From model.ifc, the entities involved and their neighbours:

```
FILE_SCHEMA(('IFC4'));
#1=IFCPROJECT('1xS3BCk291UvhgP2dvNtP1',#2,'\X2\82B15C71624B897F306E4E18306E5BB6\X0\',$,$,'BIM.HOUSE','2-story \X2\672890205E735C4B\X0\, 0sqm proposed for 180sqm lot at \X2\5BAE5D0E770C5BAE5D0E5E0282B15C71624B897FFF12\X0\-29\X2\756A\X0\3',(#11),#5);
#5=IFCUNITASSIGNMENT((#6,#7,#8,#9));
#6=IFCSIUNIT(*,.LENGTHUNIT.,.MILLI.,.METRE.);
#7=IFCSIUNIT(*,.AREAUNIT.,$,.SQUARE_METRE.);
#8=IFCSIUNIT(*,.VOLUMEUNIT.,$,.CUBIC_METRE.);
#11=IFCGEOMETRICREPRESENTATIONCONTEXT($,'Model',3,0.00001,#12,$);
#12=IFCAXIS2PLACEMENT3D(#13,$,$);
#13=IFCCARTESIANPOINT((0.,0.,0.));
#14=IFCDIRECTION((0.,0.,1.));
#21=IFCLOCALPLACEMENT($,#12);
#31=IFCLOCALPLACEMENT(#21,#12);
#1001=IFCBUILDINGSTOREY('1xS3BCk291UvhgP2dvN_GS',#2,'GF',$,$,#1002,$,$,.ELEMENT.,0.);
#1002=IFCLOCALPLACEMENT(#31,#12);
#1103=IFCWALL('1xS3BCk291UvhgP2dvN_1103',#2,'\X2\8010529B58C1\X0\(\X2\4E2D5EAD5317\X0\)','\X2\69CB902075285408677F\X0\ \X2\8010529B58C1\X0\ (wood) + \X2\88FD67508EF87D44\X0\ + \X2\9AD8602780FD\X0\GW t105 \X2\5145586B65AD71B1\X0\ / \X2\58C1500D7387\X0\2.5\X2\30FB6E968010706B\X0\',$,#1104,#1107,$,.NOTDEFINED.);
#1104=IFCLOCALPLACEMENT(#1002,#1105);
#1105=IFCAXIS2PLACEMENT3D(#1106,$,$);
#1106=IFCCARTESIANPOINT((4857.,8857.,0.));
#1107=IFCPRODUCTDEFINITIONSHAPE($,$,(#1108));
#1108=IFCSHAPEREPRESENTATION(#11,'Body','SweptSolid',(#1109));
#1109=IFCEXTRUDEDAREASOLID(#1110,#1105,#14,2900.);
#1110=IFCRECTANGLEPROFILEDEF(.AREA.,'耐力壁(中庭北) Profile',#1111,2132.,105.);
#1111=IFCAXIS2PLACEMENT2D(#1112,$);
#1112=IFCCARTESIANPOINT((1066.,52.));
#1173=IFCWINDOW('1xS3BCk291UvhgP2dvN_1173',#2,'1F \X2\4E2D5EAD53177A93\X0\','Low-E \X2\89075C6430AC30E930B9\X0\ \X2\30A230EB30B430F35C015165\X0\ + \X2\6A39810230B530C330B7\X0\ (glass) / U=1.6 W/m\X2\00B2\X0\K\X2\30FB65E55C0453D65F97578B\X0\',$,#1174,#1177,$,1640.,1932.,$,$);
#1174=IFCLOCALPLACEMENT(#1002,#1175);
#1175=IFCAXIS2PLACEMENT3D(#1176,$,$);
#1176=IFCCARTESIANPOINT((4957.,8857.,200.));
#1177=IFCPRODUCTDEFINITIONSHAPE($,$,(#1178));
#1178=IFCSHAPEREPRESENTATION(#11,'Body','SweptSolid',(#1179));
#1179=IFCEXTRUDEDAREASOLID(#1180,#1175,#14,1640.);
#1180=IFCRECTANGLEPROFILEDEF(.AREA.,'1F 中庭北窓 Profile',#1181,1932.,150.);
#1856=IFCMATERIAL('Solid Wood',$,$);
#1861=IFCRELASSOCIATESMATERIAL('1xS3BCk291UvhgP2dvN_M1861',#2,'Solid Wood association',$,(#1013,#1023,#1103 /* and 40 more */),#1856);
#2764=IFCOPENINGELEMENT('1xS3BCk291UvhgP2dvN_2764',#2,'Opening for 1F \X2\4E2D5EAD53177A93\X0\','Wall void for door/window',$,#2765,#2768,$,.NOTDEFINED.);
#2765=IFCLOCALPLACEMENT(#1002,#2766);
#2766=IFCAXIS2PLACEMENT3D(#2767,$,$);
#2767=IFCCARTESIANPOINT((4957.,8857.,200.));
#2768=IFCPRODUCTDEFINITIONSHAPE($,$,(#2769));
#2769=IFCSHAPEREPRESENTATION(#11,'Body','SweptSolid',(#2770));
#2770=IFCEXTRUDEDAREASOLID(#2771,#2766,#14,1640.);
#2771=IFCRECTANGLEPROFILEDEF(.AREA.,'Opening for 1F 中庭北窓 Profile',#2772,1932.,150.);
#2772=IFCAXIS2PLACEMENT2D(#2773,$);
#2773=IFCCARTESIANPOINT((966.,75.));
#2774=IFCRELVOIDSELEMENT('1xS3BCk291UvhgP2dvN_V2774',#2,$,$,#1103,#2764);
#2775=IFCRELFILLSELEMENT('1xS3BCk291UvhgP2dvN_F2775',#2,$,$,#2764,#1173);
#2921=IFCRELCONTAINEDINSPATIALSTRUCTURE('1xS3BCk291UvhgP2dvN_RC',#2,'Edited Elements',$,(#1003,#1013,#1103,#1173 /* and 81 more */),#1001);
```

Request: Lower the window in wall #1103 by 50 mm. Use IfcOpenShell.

```python
import numpy as np
import ifcopenshell
import ifcopenshell.api.geometry
import ifcopenshell.util.placement
import ifcopenshell.util.unit

model = ifcopenshell.open("model.ifc")
unit_scale = ifcopenshell.util.unit.calculate_unit_scale(model)

window = model.by_guid("1xS3BCk291UvhgP2dvN_1173")
opening = window.FillsVoids[0].RelatingOpeningElement
dz = -50.0

shift = np.array([0.0, 0.0, dz])
# The window is not placed relative to its opening, so move both.
for product in (opening, window):
    matrix = ifcopenshell.util.placement.get_local_placement(product.ObjectPlacement)
    matrix[:3, 3] += shift
    ifcopenshell.api.geometry.edit_object_placement(model, product=product, matrix=matrix, is_si=False)

print(f"moved by {dz * unit_scale:+.3f} m")

model.write("model_updated.ifc")
```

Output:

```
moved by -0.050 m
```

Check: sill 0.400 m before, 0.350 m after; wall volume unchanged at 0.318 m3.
